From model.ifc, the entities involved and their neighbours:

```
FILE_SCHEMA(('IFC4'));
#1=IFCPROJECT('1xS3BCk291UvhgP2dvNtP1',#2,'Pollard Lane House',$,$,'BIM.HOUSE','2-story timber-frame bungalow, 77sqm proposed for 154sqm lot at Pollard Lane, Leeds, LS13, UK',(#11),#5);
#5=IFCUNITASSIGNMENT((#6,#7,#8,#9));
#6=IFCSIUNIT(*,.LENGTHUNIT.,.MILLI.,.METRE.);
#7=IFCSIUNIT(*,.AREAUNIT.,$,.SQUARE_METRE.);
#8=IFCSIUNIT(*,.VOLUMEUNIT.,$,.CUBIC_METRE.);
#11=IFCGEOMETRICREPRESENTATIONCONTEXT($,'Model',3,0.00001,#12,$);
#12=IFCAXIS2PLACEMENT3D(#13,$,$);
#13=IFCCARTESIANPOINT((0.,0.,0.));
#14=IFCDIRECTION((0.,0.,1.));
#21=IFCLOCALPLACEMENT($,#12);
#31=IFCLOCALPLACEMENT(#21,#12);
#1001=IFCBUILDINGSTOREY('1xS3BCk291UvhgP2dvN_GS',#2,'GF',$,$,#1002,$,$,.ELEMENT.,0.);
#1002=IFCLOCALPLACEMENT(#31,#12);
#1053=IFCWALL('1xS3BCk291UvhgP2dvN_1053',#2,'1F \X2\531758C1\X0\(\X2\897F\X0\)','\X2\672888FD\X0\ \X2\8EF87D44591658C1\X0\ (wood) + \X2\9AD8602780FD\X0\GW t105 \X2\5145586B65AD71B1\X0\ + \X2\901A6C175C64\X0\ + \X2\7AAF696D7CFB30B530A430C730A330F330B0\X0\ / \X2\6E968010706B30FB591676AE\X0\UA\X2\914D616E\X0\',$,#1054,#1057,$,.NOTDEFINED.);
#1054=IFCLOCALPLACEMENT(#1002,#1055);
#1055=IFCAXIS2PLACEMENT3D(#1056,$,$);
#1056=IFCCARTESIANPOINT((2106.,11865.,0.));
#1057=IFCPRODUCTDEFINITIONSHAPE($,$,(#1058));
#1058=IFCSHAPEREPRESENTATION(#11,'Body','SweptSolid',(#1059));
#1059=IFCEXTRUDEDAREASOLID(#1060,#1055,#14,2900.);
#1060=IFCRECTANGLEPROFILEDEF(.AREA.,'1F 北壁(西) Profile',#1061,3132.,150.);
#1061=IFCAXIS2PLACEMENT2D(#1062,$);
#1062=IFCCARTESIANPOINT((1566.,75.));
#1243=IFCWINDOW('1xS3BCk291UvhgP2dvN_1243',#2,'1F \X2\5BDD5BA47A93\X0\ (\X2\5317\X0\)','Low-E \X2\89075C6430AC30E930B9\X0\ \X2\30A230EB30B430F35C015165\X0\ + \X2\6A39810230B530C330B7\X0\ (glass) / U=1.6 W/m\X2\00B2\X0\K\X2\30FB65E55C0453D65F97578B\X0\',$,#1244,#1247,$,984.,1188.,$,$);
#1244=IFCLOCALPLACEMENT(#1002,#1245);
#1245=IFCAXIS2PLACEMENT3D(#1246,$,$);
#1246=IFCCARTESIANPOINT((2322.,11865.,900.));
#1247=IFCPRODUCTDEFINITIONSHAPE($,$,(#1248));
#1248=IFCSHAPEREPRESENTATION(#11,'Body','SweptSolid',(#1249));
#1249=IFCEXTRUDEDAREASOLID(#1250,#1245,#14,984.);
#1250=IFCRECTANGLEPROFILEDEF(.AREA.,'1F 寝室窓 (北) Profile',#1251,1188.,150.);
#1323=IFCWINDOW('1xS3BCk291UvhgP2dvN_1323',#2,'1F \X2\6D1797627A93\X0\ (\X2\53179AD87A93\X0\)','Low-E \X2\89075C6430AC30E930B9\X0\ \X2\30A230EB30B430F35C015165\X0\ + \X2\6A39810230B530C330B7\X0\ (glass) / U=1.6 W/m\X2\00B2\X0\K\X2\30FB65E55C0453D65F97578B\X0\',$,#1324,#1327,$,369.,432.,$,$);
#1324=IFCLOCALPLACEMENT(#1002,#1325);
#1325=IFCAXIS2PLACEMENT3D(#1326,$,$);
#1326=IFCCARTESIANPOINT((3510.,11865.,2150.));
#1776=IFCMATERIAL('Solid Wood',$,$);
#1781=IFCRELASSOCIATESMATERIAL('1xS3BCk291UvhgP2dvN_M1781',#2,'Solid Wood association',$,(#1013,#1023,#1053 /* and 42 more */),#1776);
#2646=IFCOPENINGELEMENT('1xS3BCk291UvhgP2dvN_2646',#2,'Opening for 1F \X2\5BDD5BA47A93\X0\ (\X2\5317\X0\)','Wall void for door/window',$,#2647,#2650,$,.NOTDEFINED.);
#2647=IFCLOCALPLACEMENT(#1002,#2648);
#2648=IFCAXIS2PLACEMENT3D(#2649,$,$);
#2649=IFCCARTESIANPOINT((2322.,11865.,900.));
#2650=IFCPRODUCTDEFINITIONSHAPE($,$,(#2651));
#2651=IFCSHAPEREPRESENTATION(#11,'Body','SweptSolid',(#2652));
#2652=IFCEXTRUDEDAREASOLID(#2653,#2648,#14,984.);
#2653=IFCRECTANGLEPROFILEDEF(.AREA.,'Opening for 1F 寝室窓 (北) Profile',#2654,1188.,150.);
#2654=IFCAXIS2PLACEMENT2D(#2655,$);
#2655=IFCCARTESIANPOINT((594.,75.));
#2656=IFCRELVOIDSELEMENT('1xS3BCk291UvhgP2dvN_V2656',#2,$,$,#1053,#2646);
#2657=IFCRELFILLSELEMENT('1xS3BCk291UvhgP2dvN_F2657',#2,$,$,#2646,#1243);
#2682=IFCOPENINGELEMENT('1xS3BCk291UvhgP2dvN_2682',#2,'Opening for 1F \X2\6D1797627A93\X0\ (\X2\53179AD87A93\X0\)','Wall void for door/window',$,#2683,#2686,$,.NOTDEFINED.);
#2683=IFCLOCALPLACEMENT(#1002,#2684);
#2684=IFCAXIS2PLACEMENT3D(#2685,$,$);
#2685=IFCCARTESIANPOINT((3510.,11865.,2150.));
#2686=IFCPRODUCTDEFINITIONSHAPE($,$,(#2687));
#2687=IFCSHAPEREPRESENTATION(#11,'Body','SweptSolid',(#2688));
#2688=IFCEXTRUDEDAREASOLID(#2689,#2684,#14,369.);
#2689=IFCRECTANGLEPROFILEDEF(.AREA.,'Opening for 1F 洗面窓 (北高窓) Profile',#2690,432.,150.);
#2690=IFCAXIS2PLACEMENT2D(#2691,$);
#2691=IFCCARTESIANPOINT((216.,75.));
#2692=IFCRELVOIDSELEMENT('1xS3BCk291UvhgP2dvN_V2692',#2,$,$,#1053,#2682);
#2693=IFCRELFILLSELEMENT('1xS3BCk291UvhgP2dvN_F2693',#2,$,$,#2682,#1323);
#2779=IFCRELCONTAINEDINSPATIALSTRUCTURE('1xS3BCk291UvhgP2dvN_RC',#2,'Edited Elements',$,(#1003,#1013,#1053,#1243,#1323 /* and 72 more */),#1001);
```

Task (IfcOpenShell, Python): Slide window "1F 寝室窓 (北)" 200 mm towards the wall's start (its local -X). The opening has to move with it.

```python
import ifcopenshell
import ifcopenshell.api.geometry
import ifcopenshell.util.placement
import ifcopenshell.util.unit

model = ifcopenshell.open("model.ifc")
unit_scale = ifcopenshell.util.unit.calculate_unit_scale(model)

window = model.by_id(1243)
opening = window.FillsVoids[0].RelatingOpeningElement
wall = opening.VoidsElements[0].RelatingBuildingElement

wall_matrix = ifcopenshell.util.placement.get_local_placement(wall.ObjectPlacement)
shift = wall_matrix[:3, 0] * -0.2 / unit_scale
before = ifcopenshell.util.placement.get_local_placement(window.ObjectPlacement)[:3, 3].copy()

# The window is not placed relative to its opening, so move both.
for product in (opening, window):
    matrix = ifcopenshell.util.placement.get_local_placement(product.ObjectPlacement)
    matrix[:3, 3] += shift
    ifcopenshell.api.geometry.edit_object_placement(model, product=product, matrix=matrix, is_si=False)

after = ifcopenshell.util.placement.get_local_placement(window.ObjectPlacement)[:3, 3]
print("window moved by", (after - before).round(3) + 0.0)

model.write("model_edited.ifc")
```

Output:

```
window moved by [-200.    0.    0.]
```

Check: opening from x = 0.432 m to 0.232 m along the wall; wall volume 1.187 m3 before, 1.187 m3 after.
